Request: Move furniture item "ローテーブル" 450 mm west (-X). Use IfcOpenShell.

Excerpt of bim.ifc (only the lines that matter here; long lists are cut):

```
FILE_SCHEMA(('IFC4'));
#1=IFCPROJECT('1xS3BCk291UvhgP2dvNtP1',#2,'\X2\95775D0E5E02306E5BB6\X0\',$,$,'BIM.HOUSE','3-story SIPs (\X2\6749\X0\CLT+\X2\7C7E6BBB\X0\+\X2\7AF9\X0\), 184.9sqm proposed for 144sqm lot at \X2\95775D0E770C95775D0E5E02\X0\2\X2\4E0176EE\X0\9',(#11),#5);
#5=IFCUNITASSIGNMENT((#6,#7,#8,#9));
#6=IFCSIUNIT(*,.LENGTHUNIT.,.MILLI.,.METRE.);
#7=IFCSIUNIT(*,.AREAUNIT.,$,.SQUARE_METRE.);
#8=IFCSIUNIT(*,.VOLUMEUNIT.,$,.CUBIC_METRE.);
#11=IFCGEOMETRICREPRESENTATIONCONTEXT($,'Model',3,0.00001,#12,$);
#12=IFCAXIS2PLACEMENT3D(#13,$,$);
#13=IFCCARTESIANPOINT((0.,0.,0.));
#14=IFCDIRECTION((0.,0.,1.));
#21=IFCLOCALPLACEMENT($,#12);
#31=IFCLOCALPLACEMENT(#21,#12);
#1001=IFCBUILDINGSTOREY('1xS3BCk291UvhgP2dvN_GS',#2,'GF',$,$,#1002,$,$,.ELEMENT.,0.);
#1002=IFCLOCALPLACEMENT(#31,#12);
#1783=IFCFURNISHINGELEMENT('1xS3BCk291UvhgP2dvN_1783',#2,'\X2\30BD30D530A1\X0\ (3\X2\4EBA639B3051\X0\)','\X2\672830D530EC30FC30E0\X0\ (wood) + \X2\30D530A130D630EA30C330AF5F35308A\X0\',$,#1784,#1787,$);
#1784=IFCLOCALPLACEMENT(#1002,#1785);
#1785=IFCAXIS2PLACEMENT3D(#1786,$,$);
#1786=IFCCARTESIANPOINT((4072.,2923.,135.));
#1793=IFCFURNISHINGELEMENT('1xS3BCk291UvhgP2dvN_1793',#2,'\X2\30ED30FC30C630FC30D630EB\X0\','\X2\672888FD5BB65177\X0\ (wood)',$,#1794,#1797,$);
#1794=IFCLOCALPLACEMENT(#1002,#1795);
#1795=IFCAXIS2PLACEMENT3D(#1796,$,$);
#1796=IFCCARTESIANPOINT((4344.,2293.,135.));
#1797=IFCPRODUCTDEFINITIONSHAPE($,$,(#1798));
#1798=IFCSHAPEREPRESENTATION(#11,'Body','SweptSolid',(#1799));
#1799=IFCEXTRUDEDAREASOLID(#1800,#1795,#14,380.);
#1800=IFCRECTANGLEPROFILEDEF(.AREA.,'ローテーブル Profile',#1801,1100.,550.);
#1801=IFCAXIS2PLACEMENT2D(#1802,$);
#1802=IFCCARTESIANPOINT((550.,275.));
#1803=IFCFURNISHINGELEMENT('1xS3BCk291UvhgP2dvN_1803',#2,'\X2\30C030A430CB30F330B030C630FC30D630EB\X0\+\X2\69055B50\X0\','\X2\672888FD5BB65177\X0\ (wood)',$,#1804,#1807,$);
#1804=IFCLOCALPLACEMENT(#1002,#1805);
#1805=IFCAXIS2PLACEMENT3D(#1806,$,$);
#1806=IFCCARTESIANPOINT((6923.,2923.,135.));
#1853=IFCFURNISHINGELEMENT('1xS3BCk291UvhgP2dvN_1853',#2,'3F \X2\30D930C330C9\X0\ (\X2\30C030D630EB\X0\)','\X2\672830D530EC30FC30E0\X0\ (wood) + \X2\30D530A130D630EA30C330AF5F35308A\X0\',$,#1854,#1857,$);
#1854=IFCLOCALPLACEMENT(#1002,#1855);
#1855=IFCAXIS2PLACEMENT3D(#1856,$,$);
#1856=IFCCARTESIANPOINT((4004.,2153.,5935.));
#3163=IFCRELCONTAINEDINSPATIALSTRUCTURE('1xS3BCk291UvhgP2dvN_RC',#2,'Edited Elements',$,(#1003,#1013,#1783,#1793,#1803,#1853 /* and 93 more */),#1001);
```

```python
import ifcopenshell
import ifcopenshell.api.geometry
import ifcopenshell.util.placement

model = ifcopenshell.open("bim.ifc")

item = model.by_id(1793)
matrix = ifcopenshell.util.placement.get_local_placement(item.ObjectPlacement)
matrix[0, 3] -= 450.0
ifcopenshell.api.geometry.edit_object_placement(model, product=item, matrix=matrix, is_si=False)

print(ifcopenshell.util.placement.get_local_placement(item.ObjectPlacement).round(3) + 0.0)

model.write("bim_v2.ifc")
```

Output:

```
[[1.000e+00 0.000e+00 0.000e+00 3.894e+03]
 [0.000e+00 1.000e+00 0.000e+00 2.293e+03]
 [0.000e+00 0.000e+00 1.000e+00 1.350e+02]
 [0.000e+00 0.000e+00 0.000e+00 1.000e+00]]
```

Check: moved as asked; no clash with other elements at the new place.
